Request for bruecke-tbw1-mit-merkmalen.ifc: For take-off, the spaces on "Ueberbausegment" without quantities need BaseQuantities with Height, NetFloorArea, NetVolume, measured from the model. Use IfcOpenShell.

First a look at what the model holds.

```python
import ifcopenshell
import ifcopenshell.util.element
import ifcopenshell.util.unit

model = ifcopenshell.open("bruecke-tbw1-mit-merkmalen.ifc")
print(model.schema)
for unit_type in ("LENGTHUNIT", "AREAUNIT", "VOLUMEUNIT"):
    print(unit_type, ifcopenshell.util.unit.calculate_unit_scale(model, unit_type))
storey = next(s for s in model.by_type("IfcBuildingStorey") if s.Name == "Ueberbausegment")
spaces = [e for e in ifcopenshell.util.element.get_decomposition(storey) if e.is_a("IfcSpace")]
for e in sorted(spaces, key=lambda e: e.id()):
    print(e.id(), e.is_a(), e.Name, list(ifcopenshell.util.element.get_psets(e, qtos_only=True)), sep=" | ")
```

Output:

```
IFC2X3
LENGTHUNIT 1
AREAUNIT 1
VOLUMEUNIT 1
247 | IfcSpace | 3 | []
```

```python
import ifcopenshell
import ifcopenshell.api.pset
import ifcopenshell.geom
import ifcopenshell.util.element
import ifcopenshell.util.shape
import ifcopenshell.util.unit

model = ifcopenshell.open("bruecke-tbw1-mit-merkmalen.ifc")
unit_scale = ifcopenshell.util.unit.calculate_unit_scale(model)
area_scale = ifcopenshell.util.unit.calculate_unit_scale(model, "AREAUNIT")
volume_scale = ifcopenshell.util.unit.calculate_unit_scale(model, "VOLUMEUNIT")
settings = ifcopenshell.geom.settings()

storey = next(s for s in model.by_type("IfcBuildingStorey") if s.Name == "Ueberbausegment")
spaces = [e for e in ifcopenshell.util.element.get_decomposition(storey) if e.is_a("IfcSpace")]

for e in sorted(spaces, key=lambda e: e.id()):
    if ifcopenshell.util.element.get_psets(e, qtos_only=True, should_inherit=False):
        continue
    # Geometry comes back in metres, in the element's own axes.
    shape = ifcopenshell.geom.create_shape(settings, e)
    values = {
        "Height": ifcopenshell.util.shape.get_z(shape.geometry) / unit_scale,
        "NetFloorArea": ifcopenshell.util.shape.get_footprint_area(shape.geometry) / area_scale,
        "NetVolume": ifcopenshell.util.shape.get_volume(shape.geometry) / volume_scale,
    }
    qto = ifcopenshell.api.pset.add_qto(model, product=e, name="BaseQuantities")
    ifcopenshell.api.pset.edit_qto(model, qto=qto, properties=values)
    print(e.id(), {k: round(v, 3) for k, v in values.items()})

model.write("bruecke-tbw1-mit-merkmalen_edited.ifc")
```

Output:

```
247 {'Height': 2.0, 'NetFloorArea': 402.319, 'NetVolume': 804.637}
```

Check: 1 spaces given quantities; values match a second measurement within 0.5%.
